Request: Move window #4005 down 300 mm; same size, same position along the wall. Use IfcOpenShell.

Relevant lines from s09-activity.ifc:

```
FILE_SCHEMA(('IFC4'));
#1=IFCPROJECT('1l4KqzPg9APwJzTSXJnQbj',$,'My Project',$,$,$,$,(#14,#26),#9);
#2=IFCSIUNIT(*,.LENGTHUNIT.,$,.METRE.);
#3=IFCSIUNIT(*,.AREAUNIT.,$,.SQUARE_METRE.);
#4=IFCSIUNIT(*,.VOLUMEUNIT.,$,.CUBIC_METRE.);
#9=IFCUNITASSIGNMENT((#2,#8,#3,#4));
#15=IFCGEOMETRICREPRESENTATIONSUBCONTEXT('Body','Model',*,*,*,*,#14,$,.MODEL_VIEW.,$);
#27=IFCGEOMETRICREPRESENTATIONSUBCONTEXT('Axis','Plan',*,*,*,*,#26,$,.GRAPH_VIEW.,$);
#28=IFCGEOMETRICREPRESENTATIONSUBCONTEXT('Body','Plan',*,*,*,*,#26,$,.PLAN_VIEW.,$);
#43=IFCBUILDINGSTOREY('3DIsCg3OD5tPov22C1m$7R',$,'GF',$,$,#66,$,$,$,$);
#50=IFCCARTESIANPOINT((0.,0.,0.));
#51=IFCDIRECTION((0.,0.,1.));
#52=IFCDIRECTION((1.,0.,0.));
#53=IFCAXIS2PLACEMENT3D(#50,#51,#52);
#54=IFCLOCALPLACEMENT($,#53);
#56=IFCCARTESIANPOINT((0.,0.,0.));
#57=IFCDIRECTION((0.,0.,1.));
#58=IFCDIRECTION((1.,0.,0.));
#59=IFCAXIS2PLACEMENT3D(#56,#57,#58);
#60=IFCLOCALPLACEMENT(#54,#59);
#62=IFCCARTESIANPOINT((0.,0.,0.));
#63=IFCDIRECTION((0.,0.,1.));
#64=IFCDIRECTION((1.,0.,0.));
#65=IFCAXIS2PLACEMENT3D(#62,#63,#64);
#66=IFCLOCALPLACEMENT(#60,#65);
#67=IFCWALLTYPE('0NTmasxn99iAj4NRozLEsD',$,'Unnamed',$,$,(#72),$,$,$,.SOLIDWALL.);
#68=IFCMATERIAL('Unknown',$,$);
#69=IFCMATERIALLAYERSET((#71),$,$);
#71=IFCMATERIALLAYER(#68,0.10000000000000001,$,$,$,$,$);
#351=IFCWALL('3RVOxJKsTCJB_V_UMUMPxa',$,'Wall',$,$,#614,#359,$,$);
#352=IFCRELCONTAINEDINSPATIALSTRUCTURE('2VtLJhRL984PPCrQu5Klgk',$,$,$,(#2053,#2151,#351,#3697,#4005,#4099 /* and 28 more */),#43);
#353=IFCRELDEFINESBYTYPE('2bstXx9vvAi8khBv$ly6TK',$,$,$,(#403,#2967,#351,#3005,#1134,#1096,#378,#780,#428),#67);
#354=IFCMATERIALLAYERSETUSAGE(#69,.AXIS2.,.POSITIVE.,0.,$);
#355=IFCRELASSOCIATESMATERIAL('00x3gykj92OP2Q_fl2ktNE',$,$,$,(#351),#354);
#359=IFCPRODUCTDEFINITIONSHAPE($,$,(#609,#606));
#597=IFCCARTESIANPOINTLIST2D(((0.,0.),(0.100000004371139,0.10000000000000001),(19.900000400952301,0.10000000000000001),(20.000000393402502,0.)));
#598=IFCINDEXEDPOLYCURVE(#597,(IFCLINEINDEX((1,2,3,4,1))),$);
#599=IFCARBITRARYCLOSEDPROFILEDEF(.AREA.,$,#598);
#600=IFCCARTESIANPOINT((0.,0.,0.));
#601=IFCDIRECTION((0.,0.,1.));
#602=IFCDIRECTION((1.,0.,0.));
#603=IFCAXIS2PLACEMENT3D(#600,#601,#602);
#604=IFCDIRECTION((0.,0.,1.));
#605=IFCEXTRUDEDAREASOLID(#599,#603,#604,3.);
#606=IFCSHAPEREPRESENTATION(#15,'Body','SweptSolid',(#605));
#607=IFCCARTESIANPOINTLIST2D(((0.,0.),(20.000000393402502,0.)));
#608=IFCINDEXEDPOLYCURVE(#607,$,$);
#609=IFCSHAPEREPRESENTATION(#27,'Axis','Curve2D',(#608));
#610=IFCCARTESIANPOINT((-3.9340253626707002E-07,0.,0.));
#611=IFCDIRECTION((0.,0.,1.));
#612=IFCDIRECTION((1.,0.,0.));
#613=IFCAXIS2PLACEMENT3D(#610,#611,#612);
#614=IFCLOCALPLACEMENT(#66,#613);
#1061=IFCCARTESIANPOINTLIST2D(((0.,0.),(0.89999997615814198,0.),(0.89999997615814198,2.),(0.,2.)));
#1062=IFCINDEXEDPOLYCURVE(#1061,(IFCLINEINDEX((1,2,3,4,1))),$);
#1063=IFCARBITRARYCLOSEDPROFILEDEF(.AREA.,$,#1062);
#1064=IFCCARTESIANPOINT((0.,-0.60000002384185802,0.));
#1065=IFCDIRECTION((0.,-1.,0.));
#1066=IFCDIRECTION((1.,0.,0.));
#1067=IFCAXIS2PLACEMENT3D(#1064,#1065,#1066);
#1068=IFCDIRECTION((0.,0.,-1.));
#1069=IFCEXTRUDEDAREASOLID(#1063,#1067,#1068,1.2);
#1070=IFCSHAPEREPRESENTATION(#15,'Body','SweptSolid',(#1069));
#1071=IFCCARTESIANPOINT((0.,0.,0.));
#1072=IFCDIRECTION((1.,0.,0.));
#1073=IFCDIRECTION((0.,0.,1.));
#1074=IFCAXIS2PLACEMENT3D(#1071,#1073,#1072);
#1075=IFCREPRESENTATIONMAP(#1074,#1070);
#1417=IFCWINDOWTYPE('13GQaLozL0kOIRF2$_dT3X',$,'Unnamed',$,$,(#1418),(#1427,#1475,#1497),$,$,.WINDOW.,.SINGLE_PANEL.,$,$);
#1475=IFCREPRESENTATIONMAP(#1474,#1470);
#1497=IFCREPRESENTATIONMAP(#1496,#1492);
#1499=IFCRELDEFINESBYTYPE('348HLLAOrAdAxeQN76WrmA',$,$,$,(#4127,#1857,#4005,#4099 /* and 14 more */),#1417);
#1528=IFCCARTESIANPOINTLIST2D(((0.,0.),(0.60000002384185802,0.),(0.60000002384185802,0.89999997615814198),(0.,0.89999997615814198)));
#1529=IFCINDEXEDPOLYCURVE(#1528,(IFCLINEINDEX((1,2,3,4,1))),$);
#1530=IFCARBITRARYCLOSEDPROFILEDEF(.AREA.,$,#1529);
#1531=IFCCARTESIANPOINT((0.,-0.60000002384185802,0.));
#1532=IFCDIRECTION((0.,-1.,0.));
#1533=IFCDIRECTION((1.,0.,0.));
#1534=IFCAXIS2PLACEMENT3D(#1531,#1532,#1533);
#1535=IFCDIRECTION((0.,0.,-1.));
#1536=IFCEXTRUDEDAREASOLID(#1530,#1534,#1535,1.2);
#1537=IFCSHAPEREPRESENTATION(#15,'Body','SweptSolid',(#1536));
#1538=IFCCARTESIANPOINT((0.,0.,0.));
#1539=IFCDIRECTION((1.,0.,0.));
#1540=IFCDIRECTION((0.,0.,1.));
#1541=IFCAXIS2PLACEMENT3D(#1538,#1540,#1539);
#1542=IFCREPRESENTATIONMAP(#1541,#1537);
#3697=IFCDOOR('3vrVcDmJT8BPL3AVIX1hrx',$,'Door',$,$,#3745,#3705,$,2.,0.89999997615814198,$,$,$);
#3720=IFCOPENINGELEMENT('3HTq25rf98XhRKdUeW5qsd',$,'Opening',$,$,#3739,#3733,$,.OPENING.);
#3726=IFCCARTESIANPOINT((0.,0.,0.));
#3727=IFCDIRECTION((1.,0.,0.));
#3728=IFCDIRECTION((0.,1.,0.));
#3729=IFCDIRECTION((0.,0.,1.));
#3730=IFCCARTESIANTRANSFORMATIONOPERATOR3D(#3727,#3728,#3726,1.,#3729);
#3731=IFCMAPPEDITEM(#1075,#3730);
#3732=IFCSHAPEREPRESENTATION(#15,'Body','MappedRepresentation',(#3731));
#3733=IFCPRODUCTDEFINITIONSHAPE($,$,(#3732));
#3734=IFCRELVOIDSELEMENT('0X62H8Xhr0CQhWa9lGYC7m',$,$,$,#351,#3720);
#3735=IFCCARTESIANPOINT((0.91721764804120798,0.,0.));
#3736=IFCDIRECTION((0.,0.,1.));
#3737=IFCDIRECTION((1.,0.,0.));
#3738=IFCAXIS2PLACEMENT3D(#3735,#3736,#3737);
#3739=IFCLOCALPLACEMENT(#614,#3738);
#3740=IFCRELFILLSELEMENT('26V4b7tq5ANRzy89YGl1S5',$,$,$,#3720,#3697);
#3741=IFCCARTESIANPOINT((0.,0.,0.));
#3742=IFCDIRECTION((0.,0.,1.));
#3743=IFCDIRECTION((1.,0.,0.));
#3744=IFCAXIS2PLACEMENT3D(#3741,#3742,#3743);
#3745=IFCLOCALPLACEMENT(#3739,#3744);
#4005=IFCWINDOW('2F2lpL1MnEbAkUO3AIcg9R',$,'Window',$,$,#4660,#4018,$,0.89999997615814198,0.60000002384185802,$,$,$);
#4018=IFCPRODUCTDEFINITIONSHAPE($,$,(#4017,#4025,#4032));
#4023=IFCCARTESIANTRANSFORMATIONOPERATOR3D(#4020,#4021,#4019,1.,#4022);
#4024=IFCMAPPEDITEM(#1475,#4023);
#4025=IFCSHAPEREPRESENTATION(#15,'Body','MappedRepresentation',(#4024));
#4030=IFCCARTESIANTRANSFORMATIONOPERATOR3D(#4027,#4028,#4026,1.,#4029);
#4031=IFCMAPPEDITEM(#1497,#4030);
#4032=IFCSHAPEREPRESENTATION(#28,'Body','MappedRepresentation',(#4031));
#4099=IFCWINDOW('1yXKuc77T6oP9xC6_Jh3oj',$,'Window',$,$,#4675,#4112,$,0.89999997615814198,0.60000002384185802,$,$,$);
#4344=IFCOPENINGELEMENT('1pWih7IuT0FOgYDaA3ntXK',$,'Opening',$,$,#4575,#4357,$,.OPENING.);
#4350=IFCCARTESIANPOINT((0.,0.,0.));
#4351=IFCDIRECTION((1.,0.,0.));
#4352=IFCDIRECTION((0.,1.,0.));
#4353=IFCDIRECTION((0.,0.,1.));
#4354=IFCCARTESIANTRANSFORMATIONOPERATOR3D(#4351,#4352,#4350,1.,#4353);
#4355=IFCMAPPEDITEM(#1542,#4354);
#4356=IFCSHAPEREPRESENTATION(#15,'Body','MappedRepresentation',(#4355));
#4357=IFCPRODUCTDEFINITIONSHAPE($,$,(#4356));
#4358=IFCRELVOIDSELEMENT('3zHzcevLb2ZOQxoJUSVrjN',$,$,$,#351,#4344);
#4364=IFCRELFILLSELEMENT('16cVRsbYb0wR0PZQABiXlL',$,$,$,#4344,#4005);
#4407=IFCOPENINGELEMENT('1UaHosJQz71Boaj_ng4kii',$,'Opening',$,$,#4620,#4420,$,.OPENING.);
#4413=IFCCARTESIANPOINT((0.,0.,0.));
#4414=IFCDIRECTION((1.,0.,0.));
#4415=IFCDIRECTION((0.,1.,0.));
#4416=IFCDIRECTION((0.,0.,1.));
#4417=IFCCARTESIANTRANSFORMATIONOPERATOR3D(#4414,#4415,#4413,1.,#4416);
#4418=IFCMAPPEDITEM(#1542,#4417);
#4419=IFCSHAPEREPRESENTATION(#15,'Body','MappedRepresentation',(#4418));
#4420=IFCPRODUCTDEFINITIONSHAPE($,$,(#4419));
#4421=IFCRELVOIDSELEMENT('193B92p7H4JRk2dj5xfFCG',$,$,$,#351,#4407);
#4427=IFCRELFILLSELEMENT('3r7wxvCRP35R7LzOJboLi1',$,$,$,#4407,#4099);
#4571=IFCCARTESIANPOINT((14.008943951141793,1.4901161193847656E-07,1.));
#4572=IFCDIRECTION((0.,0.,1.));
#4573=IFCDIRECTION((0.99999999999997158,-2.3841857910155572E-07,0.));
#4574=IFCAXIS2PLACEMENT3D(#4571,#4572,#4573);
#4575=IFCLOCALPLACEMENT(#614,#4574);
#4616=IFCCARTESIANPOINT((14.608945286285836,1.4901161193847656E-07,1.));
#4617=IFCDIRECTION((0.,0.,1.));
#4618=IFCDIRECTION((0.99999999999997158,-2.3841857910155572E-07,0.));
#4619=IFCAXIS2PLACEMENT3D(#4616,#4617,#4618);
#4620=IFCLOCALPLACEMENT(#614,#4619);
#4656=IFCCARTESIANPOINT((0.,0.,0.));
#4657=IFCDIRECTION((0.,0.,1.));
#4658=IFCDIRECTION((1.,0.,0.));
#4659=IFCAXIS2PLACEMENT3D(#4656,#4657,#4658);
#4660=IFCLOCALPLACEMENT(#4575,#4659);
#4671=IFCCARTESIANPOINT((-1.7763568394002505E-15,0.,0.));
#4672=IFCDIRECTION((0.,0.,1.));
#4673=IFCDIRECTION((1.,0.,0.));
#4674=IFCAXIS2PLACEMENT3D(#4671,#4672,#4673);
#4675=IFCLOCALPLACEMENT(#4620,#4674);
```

```python
import numpy as np
import ifcopenshell
import ifcopenshell.api.geometry
import ifcopenshell.util.placement
import ifcopenshell.util.unit

model = ifcopenshell.open("s09-activity.ifc")
unit_scale = ifcopenshell.util.unit.calculate_unit_scale(model)

window = model.by_id(4005)
opening = window.FillsVoids[0].RelatingOpeningElement
dz = -0.3

shift = np.array([0.0, 0.0, dz])
# The window is placed relative to its opening, so it follows when the opening moves.
matrix = ifcopenshell.util.placement.get_local_placement(opening.ObjectPlacement)
matrix[:3, 3] += shift
ifcopenshell.api.geometry.edit_object_placement(
    model, product=opening, matrix=matrix, is_si=False, should_transform_children=True
)

print(f"moved by {dz * unit_scale:+.3f} m")

model.write("s09-activity_edited.ifc")
```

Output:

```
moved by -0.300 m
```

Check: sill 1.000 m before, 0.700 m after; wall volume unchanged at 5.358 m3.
